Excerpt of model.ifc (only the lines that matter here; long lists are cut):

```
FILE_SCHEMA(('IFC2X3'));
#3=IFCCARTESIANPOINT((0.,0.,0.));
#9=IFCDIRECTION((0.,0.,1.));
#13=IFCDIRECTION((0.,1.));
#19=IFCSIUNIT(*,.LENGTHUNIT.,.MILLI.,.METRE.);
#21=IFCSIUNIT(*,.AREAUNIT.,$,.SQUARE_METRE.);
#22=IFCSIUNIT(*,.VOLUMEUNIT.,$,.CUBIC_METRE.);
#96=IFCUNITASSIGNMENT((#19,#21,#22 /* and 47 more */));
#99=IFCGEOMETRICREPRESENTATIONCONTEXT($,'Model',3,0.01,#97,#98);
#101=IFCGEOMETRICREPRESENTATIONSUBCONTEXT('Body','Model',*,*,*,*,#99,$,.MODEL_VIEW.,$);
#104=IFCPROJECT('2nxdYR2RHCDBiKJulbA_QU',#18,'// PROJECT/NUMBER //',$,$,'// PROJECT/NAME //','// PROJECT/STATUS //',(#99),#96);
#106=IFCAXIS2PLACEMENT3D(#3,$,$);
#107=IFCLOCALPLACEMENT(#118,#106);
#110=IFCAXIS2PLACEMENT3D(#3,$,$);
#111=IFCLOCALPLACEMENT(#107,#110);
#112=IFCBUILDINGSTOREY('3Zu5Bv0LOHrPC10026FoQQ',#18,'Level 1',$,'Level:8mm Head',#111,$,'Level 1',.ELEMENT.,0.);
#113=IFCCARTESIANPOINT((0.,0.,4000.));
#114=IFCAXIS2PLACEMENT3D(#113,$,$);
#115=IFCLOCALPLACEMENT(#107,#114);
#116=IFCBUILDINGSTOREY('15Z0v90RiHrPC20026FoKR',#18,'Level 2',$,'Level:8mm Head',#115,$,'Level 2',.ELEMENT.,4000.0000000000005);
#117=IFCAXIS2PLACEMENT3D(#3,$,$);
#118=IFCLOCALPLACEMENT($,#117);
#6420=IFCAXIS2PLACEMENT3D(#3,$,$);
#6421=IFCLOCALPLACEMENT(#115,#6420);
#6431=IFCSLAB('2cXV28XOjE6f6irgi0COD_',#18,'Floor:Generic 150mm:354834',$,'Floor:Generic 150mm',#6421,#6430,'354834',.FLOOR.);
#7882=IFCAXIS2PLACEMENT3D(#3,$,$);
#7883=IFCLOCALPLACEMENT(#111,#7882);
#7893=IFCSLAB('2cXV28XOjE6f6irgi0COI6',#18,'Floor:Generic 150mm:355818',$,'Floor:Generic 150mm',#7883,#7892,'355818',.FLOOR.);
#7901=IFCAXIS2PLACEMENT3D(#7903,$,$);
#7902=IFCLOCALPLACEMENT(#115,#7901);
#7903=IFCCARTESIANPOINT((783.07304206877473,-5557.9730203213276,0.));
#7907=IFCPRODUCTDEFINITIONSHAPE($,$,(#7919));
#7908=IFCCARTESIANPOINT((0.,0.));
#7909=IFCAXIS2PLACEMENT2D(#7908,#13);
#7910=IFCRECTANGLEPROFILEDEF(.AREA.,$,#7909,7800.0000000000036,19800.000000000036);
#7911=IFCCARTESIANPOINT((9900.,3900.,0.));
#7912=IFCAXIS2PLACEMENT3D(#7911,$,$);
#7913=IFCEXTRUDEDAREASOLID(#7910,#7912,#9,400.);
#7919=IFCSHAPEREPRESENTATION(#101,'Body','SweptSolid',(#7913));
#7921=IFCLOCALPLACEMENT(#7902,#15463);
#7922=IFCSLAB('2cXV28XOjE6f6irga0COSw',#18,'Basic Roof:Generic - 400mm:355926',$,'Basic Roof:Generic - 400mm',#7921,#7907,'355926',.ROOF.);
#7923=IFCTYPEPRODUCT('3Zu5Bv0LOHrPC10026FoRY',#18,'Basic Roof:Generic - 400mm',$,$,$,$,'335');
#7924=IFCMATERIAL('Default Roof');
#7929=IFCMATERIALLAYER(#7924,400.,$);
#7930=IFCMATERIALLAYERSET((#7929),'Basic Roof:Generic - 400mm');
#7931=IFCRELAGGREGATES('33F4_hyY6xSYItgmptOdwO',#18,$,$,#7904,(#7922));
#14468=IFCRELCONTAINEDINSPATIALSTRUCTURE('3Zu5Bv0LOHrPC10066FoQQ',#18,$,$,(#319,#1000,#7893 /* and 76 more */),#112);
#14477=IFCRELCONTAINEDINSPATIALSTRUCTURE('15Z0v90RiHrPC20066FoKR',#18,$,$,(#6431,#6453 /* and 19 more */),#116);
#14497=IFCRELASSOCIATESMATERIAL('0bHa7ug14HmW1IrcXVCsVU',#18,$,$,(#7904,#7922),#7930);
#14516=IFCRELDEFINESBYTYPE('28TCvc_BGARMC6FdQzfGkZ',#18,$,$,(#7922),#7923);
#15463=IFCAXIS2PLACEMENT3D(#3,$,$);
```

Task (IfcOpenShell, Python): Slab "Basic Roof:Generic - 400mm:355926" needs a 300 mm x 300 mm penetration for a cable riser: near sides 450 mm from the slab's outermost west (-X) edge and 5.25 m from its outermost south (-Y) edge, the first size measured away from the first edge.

```python
import numpy as np
import ifcopenshell
import ifcopenshell.api.feature
import ifcopenshell.api.geometry
import ifcopenshell.api.root
import ifcopenshell.geom
import ifcopenshell.util.placement
import ifcopenshell.util.representation
import ifcopenshell.util.shape
import ifcopenshell.util.unit

model = ifcopenshell.open("model.ifc")
unit_scale = ifcopenshell.util.unit.calculate_unit_scale(model)
settings = ifcopenshell.geom.settings()


def volume(element):
    """Net volume in cubic metres, openings subtracted."""
    shape = ifcopenshell.geom.create_shape(settings, element)
    return ifcopenshell.util.shape.get_volume(shape.geometry)


slab = model.by_id(7922)
before = volume(slab)

# Extent in the slab's own axes, in metres. The edges named are its -X and -Y sides.
slab_shape = ifcopenshell.geom.create_shape(settings, slab)
vertices = ifcopenshell.util.shape.get_vertices(slab_shape.geometry)
x_min, y_min, bottom = vertices.min(axis=0)
top = vertices[:, 2].max()

opening = ifcopenshell.api.root.create_entity(model, ifc_class="IfcOpeningElement", name="Cable riser opening")
context = ifcopenshell.util.representation.get_context(model, "Model", "Body", "MODEL_VIEW")
width, depth = 0.3, 0.3
outline = [(0.0, 0.0), (width, 0.0), (width, depth), (0.0, depth), (0.0, 0.0)]
# Overshoot both faces by 50 mm so the cut is clean.
shape = ifcopenshell.api.geometry.add_slab_representation(
    model, context=context, depth=top - bottom + 0.1, polyline=outline
)
ifcopenshell.api.geometry.assign_representation(model, product=opening, representation=shape)

matrix = ifcopenshell.util.placement.get_local_placement(slab.ObjectPlacement)
matrix[:, 3] = matrix @ np.append(np.array([x_min + 0.45, y_min + 5.25, bottom - 0.05]) / unit_scale, 1.0)
ifcopenshell.api.geometry.edit_object_placement(model, product=opening, matrix=matrix, is_si=False)
ifcopenshell.api.feature.add_feature(model, feature=opening, element=slab)

after = volume(slab)

print(f"slab volume {before:.3f} -> {after:.3f} m3")

model.write("model-out.ifc")
```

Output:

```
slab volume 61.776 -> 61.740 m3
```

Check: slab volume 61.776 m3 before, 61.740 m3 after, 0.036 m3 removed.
